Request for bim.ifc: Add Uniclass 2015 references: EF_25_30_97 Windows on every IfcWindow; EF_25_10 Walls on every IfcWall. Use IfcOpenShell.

First a look at what the model holds.

```python
import ifcopenshell

model = ifcopenshell.open("bim.ifc")
print(model.schema)
print("classifications:", [c.Name for c in model.by_type("IfcClassification")])
for ifc_class in ("IfcDoor", "IfcRoof", "IfcStair", "IfcWall", "IfcWindow"):
    print(ifc_class, len(model.by_type(ifc_class)))
```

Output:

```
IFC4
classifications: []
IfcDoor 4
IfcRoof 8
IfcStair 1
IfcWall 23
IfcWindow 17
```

```python
import ifcopenshell
import ifcopenshell.api.classification

model = ifcopenshell.open("bim.ifc")

system = ifcopenshell.api.classification.add_classification(model, classification="Uniclass 2015")

codes = {
    "IfcWindow": ("EF_25_30_97", "Windows"),
    "IfcWall": ("EF_25_10", "Walls"),
}
for ifc_class, (code, name) in codes.items():
    products = model.by_type(ifc_class)
    ifcopenshell.api.classification.add_reference(
        model, products=products, classification=system, identification=code, name=name
    )
    print(code, len(products))

model.write("bim_rev.ifc")
```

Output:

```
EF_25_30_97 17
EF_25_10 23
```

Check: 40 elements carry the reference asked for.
